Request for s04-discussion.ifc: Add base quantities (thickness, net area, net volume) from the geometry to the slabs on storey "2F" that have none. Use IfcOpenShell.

First a look at what the model holds.

```python
import ifcopenshell
import ifcopenshell.util.element
import ifcopenshell.util.unit

model = ifcopenshell.open("s04-discussion.ifc")
print(model.schema)
for unit_type in ("LENGTHUNIT", "AREAUNIT", "VOLUMEUNIT"):
    print(unit_type, ifcopenshell.util.unit.calculate_unit_scale(model, unit_type))
storey = next(s for s in model.by_type("IfcBuildingStorey") if s.Name == "2F")
slabs = [e for e in ifcopenshell.util.element.get_decomposition(storey) if e.is_a("IfcSlab")]
for e in sorted(slabs, key=lambda e: e.id()):
    print(e.id(), e.is_a(), e.Name, list(ifcopenshell.util.element.get_psets(e, qtos_only=True)), sep=" | ")
```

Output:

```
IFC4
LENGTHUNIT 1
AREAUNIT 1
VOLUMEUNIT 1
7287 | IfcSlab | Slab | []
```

```python
import ifcopenshell
import ifcopenshell.api.pset
import ifcopenshell.geom
import ifcopenshell.util.element
import ifcopenshell.util.shape
import ifcopenshell.util.unit

model = ifcopenshell.open("s04-discussion.ifc")
unit_scale = ifcopenshell.util.unit.calculate_unit_scale(model)
area_scale = ifcopenshell.util.unit.calculate_unit_scale(model, "AREAUNIT")
volume_scale = ifcopenshell.util.unit.calculate_unit_scale(model, "VOLUMEUNIT")
settings = ifcopenshell.geom.settings()

storey = next(s for s in model.by_type("IfcBuildingStorey") if s.Name == "2F")
slabs = [e for e in ifcopenshell.util.element.get_decomposition(storey) if e.is_a("IfcSlab")]

for e in sorted(slabs, key=lambda e: e.id()):
    if ifcopenshell.util.element.get_psets(e, qtos_only=True, should_inherit=False):
        continue
    # Geometry comes back in metres, in the element's own axes.
    shape = ifcopenshell.geom.create_shape(settings, e)
    values = {
        "Width": ifcopenshell.util.shape.get_z(shape.geometry) / unit_scale,
        "NetArea": ifcopenshell.util.shape.get_footprint_area(shape.geometry) / area_scale,
        "NetVolume": ifcopenshell.util.shape.get_volume(shape.geometry) / volume_scale,
    }
    qto = ifcopenshell.api.pset.add_qto(model, product=e, name="Qto_SlabBaseQuantities")
    ifcopenshell.api.pset.edit_qto(model, qto=qto, properties=values)
    print(e.id(), {k: round(v, 3) for k, v in values.items()})

model.write("s04-discussion_updated.ifc")
```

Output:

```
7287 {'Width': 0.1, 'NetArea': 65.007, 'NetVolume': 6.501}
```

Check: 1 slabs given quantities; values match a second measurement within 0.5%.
